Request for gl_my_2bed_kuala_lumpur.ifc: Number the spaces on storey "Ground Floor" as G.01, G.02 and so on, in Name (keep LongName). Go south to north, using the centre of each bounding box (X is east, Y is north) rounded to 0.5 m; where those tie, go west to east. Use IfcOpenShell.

First a look at what the model holds.

```python
import ifcopenshell
import ifcopenshell.util.element
import ifcopenshell.util.placement

model = ifcopenshell.open("gl_my_2bed_kuala_lumpur.ifc")
print(model.schema)
storey = next(s for s in model.by_type("IfcBuildingStorey") if s.Name == "Ground Floor")
spaces = [e for e in ifcopenshell.util.element.get_decomposition(storey) if e.is_a("IfcSpace")]
for e in sorted(spaces, key=lambda e: e.id()):
    origin = ifcopenshell.util.placement.get_local_placement(e.ObjectPlacement)[:3, 3]
    print(e.id(), e.Name, e.LongName, origin.round(2) + 0.0, sep=" | ")
```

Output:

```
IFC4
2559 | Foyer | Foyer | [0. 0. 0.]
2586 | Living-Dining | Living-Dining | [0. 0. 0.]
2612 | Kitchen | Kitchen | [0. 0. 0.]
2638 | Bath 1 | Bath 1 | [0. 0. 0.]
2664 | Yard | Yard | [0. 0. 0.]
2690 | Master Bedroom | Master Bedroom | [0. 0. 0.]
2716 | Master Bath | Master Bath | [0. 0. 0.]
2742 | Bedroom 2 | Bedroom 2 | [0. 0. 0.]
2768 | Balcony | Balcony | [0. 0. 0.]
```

```python
import ifcopenshell
import ifcopenshell.geom
import ifcopenshell.util.element
import ifcopenshell.util.shape

model = ifcopenshell.open("gl_my_2bed_kuala_lumpur.ifc")
settings = ifcopenshell.geom.settings()
settings.set("use-world-coords", True)


def centre(element):
    shape = ifcopenshell.geom.create_shape(settings, element)
    return ifcopenshell.util.shape.get_bbox_centroid(shape.geometry)


storey = next(s for s in model.by_type("IfcBuildingStorey") if s.Name == "Ground Floor")
spaces = [e for e in ifcopenshell.util.element.get_decomposition(storey) if e.is_a("IfcSpace")]

# Insertion points can sit at a corner or the storey origin, so sort by the geometry (in metres).
centres = {e: centre(e) for e in spaces}
spaces.sort(key=lambda e: (round(centres[e][1] / 0.5), centres[e][0]))

for i, e in enumerate(spaces, start=1):
    number = f"G.{i:02d}"
    e.Name = number
    print(e.id(), number)

model.write("gl_my_2bed_kuala_lumpur_v2.ifc")
```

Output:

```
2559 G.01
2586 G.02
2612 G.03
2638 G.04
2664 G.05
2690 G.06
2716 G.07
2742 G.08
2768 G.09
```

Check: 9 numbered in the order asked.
